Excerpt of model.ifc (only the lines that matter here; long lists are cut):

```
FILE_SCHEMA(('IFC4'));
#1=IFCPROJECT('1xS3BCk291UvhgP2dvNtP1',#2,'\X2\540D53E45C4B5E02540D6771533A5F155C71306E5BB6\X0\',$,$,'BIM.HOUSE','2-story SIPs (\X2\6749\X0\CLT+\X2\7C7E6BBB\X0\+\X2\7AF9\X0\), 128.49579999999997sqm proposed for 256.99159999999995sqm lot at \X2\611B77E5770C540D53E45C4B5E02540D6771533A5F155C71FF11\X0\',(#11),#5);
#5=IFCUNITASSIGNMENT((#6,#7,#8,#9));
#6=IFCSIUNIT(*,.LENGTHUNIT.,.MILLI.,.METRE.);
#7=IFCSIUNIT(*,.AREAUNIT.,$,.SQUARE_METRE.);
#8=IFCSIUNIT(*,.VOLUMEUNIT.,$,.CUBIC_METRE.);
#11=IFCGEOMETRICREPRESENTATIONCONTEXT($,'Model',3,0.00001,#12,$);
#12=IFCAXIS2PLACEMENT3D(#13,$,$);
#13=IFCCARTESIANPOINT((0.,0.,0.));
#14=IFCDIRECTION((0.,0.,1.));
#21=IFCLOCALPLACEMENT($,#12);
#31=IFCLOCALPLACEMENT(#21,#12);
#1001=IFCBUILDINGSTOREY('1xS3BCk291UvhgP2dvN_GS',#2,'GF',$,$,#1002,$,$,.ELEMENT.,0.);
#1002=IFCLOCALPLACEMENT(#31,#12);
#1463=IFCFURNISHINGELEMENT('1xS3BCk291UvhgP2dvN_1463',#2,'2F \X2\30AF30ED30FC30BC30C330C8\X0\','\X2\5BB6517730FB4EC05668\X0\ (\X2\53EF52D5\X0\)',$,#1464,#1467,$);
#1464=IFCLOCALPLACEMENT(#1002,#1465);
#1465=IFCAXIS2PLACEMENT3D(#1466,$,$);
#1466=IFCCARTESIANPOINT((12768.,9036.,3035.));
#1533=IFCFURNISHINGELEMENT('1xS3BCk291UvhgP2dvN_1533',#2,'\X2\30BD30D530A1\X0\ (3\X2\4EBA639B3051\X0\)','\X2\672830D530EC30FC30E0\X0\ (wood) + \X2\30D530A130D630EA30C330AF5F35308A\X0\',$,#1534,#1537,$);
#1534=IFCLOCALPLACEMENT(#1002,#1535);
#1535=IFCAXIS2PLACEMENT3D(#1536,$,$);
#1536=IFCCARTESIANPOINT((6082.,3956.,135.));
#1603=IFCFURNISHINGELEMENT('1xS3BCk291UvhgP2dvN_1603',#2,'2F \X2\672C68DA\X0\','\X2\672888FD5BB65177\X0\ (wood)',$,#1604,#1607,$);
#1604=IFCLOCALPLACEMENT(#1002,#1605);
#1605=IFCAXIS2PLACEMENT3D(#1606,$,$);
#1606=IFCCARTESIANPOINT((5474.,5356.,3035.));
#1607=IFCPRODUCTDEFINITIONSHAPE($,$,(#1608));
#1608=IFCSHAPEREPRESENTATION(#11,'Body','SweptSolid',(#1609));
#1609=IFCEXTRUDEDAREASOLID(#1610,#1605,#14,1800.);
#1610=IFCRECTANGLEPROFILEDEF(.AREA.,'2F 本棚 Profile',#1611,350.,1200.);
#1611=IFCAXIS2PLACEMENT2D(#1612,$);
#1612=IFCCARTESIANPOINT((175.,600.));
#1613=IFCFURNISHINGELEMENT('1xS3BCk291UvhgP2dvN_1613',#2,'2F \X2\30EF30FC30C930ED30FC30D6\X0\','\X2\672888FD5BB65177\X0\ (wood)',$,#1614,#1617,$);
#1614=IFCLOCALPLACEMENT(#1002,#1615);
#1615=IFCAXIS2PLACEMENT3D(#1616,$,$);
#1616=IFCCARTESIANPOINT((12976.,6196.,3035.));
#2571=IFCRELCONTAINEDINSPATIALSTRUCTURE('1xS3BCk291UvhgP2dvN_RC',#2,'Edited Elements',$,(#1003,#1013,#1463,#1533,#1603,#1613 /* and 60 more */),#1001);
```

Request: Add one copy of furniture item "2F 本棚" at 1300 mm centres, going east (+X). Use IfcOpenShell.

```python
import numpy as np
import ifcopenshell
import ifcopenshell.api.geometry
import ifcopenshell.api.root
import ifcopenshell.util.element
import ifcopenshell.util.placement
import ifcopenshell.util.unit

model = ifcopenshell.open("model.ifc")
unit_scale = ifcopenshell.util.unit.calculate_unit_scale(model)


def reuse_history(source, copy):
    """copy_class also copies each property set's owner history, people and application; keep the originals."""
    for rel in copy.IsDefinedBy:
        if rel.is_a("IfcRelDefinesByProperties") and (history := rel.RelatingPropertyDefinition.OwnerHistory):
            rel.RelatingPropertyDefinition.OwnerHistory = source.OwnerHistory
            ifcopenshell.util.element.remove_deep2(model, history)


source = model.by_guid("1xS3BCk291UvhgP2dvN_1603")
base = ifcopenshell.util.placement.get_local_placement(source.ObjectPlacement)
step = np.array([1.0, 0.0, 0.0]) * 1.3 / unit_scale

for i in range(1, 2):
    copy = ifcopenshell.api.root.copy_class(model, product=source)
    copy.Representation = ifcopenshell.util.element.copy_deep(
        model, source.Representation, exclude=["IfcGeometricRepresentationContext", "IfcRepresentationMap"]
    )
    reuse_history(source, copy)
    matrix = base.copy()
    matrix[:3, 3] += i * step
    print("added at", matrix[:3, 3].round(3) + 0.0)
    ifcopenshell.api.geometry.edit_object_placement(model, product=copy, matrix=matrix, is_si=False)

model.write("model-out.ifc")
```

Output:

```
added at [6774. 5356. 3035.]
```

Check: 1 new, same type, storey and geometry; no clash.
